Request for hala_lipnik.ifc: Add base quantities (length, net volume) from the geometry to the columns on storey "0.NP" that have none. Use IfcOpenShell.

First a look at what the model holds.

```python
import ifcopenshell
import ifcopenshell.util.element
import ifcopenshell.util.unit

model = ifcopenshell.open("hala_lipnik.ifc")
print(model.schema)
for unit_type in ("LENGTHUNIT", "AREAUNIT", "VOLUMEUNIT"):
    print(unit_type, ifcopenshell.util.unit.calculate_unit_scale(model, unit_type))
storey = next(s for s in model.by_type("IfcBuildingStorey") if s.Name == "0.NP")
columns = [e for e in ifcopenshell.util.element.get_decomposition(storey) if e.is_a("IfcColumn")]
for e in sorted(columns, key=lambda e: e.id()):
    print(e.id(), e.is_a(), e.Name, list(ifcopenshell.util.element.get_psets(e, qtos_only=True)), sep=" | ")
```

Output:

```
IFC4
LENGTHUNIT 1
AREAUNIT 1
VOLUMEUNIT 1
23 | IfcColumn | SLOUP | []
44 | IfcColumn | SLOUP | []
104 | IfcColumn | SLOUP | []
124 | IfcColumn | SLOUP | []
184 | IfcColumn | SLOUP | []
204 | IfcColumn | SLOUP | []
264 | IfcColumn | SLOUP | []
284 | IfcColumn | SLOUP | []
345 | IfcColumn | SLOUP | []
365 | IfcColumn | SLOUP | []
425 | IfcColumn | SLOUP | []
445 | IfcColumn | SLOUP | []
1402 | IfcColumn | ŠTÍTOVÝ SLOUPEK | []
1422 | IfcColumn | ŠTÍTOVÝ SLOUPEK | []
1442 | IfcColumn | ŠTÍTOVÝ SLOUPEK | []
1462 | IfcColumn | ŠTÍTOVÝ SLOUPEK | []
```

```python
import ifcopenshell
import ifcopenshell.api.pset
import ifcopenshell.geom
import ifcopenshell.util.element
import ifcopenshell.util.shape
import ifcopenshell.util.unit

model = ifcopenshell.open("hala_lipnik.ifc")
unit_scale = ifcopenshell.util.unit.calculate_unit_scale(model)
volume_scale = ifcopenshell.util.unit.calculate_unit_scale(model, "VOLUMEUNIT")
settings = ifcopenshell.geom.settings()

storey = next(s for s in model.by_type("IfcBuildingStorey") if s.Name == "0.NP")
columns = [e for e in ifcopenshell.util.element.get_decomposition(storey) if e.is_a("IfcColumn")]

for e in sorted(columns, key=lambda e: e.id()):
    if ifcopenshell.util.element.get_psets(e, qtos_only=True, should_inherit=False):
        continue
    # Geometry comes back in metres, in the element's own axes.
    shape = ifcopenshell.geom.create_shape(settings, e)
    values = {
        "Length": ifcopenshell.util.shape.get_z(shape.geometry) / unit_scale,
        "NetVolume": ifcopenshell.util.shape.get_volume(shape.geometry) / volume_scale,
    }
    qto = ifcopenshell.api.pset.add_qto(model, product=e, name="Qto_ColumnBaseQuantities")
    ifcopenshell.api.pset.edit_qto(model, qto=qto, properties=values)
    print(e.id(), {k: round(v, 3) for k, v in values.items()})

model.write("hala_lipnik_edited.ifc")
```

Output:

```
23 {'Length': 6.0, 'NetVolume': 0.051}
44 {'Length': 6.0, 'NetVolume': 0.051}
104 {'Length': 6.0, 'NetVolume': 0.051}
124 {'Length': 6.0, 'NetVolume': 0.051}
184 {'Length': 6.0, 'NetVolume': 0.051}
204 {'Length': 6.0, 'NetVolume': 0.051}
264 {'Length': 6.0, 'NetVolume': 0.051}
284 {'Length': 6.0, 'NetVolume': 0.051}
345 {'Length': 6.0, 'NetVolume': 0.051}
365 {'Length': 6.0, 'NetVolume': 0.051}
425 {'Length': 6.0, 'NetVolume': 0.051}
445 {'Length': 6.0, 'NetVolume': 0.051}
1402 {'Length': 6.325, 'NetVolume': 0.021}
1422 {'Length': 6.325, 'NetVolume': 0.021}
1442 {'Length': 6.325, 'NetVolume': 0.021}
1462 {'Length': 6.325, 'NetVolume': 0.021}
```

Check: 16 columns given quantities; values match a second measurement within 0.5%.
